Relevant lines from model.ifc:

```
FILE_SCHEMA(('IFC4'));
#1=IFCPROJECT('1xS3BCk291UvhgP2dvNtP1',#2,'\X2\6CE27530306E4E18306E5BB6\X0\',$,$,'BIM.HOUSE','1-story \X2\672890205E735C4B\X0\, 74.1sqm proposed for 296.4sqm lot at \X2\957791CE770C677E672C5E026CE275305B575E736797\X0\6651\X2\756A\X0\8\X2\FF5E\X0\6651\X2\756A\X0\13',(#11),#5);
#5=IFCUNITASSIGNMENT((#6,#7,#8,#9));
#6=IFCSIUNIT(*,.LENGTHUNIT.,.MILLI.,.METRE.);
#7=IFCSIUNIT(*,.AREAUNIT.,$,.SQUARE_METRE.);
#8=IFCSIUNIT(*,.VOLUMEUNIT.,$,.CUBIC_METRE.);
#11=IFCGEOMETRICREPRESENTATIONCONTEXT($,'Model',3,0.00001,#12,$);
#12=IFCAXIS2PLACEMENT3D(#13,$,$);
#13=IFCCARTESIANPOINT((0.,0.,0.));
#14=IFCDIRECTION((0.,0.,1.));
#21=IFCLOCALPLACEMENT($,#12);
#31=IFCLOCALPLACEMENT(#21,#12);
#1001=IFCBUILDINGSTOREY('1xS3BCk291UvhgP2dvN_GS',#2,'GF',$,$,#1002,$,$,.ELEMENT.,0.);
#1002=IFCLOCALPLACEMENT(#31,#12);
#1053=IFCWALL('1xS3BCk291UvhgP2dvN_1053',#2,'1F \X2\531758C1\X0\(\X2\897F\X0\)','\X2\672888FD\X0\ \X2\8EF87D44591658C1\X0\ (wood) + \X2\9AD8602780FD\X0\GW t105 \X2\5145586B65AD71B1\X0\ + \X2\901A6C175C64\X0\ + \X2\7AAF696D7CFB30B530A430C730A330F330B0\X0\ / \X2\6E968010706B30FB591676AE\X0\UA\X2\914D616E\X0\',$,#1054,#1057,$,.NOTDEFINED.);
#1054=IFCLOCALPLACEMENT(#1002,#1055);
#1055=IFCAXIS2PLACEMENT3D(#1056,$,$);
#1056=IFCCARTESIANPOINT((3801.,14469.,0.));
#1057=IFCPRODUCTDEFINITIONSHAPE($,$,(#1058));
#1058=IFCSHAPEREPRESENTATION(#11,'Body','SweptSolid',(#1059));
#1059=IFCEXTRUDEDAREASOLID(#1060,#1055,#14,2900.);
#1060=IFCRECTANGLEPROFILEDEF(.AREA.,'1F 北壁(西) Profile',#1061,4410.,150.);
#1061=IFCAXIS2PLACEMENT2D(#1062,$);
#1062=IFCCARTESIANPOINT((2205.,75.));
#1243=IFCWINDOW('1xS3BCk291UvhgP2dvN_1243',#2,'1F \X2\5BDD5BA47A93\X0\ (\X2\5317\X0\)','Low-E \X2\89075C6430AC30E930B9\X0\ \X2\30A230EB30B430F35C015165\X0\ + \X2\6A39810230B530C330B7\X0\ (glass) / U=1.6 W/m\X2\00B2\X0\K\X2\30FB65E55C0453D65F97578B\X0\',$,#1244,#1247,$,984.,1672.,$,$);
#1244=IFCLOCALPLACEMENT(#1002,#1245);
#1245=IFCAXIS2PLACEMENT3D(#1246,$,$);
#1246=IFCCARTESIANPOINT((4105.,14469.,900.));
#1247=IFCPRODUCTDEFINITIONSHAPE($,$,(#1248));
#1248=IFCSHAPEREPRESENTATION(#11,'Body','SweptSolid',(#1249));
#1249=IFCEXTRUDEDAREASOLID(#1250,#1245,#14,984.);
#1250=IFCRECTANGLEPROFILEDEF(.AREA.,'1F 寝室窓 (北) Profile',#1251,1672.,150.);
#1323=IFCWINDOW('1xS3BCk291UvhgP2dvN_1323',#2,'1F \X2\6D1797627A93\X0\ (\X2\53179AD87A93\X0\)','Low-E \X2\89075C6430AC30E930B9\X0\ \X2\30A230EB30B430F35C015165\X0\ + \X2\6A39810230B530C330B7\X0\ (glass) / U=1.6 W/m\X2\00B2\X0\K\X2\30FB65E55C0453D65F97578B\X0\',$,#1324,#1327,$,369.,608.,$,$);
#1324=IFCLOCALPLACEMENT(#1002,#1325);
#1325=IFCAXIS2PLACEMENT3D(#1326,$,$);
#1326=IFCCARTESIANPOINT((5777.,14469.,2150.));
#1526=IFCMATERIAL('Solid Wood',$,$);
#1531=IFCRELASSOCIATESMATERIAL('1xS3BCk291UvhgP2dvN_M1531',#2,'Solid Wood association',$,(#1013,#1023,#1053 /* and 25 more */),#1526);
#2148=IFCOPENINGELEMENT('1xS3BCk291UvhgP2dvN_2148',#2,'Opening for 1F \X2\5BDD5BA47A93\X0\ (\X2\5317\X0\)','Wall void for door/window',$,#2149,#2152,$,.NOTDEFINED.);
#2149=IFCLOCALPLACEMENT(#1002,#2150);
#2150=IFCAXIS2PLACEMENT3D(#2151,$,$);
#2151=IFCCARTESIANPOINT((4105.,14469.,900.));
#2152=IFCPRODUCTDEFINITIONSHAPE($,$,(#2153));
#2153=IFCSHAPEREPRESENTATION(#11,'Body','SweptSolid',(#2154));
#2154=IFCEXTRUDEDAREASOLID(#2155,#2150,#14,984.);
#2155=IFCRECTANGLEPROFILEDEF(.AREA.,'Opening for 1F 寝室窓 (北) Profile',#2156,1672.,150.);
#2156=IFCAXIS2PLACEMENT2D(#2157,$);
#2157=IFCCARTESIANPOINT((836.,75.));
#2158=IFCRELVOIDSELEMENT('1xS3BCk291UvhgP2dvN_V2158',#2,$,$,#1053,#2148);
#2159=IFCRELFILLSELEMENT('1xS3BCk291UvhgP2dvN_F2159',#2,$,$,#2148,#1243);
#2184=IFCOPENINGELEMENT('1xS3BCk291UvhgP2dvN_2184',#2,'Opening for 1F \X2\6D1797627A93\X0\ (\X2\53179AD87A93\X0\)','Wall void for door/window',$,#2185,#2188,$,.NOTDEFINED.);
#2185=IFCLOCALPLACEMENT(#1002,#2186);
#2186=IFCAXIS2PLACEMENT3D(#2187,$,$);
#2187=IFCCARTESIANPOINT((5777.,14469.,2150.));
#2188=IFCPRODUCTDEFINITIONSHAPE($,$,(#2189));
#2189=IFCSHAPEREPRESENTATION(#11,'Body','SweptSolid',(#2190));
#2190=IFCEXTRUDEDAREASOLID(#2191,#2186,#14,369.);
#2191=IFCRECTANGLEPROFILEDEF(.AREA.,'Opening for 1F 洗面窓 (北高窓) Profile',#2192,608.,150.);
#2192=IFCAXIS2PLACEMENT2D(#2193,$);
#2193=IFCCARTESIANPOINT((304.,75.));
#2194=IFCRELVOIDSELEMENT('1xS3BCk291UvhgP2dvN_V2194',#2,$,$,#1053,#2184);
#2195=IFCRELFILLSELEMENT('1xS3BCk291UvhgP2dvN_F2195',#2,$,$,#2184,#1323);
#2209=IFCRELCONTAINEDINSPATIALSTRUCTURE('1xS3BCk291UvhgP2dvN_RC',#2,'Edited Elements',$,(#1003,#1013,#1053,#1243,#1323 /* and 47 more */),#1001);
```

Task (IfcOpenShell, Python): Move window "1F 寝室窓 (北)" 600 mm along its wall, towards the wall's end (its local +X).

```python
import ifcopenshell
import ifcopenshell.api.geometry
import ifcopenshell.util.placement
import ifcopenshell.util.unit

model = ifcopenshell.open("model.ifc")
unit_scale = ifcopenshell.util.unit.calculate_unit_scale(model)

window = model.by_guid("1xS3BCk291UvhgP2dvN_1243")
opening = window.FillsVoids[0].RelatingOpeningElement
wall = opening.VoidsElements[0].RelatingBuildingElement

wall_matrix = ifcopenshell.util.placement.get_local_placement(wall.ObjectPlacement)
shift = wall_matrix[:3, 0] * 0.6 / unit_scale
before = ifcopenshell.util.placement.get_local_placement(window.ObjectPlacement)[:3, 3].copy()

# The window is not placed relative to its opening, so move both.
for product in (opening, window):
    matrix = ifcopenshell.util.placement.get_local_placement(product.ObjectPlacement)
    matrix[:3, 3] += shift
    ifcopenshell.api.geometry.edit_object_placement(model, product=product, matrix=matrix, is_si=False)

after = ifcopenshell.util.placement.get_local_placement(window.ObjectPlacement)[:3, 3]
print("window moved by", (after - before).round(3) + 0.0)

model.write("model-out.ifc")
```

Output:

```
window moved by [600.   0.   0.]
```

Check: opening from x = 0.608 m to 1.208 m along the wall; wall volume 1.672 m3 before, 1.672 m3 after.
